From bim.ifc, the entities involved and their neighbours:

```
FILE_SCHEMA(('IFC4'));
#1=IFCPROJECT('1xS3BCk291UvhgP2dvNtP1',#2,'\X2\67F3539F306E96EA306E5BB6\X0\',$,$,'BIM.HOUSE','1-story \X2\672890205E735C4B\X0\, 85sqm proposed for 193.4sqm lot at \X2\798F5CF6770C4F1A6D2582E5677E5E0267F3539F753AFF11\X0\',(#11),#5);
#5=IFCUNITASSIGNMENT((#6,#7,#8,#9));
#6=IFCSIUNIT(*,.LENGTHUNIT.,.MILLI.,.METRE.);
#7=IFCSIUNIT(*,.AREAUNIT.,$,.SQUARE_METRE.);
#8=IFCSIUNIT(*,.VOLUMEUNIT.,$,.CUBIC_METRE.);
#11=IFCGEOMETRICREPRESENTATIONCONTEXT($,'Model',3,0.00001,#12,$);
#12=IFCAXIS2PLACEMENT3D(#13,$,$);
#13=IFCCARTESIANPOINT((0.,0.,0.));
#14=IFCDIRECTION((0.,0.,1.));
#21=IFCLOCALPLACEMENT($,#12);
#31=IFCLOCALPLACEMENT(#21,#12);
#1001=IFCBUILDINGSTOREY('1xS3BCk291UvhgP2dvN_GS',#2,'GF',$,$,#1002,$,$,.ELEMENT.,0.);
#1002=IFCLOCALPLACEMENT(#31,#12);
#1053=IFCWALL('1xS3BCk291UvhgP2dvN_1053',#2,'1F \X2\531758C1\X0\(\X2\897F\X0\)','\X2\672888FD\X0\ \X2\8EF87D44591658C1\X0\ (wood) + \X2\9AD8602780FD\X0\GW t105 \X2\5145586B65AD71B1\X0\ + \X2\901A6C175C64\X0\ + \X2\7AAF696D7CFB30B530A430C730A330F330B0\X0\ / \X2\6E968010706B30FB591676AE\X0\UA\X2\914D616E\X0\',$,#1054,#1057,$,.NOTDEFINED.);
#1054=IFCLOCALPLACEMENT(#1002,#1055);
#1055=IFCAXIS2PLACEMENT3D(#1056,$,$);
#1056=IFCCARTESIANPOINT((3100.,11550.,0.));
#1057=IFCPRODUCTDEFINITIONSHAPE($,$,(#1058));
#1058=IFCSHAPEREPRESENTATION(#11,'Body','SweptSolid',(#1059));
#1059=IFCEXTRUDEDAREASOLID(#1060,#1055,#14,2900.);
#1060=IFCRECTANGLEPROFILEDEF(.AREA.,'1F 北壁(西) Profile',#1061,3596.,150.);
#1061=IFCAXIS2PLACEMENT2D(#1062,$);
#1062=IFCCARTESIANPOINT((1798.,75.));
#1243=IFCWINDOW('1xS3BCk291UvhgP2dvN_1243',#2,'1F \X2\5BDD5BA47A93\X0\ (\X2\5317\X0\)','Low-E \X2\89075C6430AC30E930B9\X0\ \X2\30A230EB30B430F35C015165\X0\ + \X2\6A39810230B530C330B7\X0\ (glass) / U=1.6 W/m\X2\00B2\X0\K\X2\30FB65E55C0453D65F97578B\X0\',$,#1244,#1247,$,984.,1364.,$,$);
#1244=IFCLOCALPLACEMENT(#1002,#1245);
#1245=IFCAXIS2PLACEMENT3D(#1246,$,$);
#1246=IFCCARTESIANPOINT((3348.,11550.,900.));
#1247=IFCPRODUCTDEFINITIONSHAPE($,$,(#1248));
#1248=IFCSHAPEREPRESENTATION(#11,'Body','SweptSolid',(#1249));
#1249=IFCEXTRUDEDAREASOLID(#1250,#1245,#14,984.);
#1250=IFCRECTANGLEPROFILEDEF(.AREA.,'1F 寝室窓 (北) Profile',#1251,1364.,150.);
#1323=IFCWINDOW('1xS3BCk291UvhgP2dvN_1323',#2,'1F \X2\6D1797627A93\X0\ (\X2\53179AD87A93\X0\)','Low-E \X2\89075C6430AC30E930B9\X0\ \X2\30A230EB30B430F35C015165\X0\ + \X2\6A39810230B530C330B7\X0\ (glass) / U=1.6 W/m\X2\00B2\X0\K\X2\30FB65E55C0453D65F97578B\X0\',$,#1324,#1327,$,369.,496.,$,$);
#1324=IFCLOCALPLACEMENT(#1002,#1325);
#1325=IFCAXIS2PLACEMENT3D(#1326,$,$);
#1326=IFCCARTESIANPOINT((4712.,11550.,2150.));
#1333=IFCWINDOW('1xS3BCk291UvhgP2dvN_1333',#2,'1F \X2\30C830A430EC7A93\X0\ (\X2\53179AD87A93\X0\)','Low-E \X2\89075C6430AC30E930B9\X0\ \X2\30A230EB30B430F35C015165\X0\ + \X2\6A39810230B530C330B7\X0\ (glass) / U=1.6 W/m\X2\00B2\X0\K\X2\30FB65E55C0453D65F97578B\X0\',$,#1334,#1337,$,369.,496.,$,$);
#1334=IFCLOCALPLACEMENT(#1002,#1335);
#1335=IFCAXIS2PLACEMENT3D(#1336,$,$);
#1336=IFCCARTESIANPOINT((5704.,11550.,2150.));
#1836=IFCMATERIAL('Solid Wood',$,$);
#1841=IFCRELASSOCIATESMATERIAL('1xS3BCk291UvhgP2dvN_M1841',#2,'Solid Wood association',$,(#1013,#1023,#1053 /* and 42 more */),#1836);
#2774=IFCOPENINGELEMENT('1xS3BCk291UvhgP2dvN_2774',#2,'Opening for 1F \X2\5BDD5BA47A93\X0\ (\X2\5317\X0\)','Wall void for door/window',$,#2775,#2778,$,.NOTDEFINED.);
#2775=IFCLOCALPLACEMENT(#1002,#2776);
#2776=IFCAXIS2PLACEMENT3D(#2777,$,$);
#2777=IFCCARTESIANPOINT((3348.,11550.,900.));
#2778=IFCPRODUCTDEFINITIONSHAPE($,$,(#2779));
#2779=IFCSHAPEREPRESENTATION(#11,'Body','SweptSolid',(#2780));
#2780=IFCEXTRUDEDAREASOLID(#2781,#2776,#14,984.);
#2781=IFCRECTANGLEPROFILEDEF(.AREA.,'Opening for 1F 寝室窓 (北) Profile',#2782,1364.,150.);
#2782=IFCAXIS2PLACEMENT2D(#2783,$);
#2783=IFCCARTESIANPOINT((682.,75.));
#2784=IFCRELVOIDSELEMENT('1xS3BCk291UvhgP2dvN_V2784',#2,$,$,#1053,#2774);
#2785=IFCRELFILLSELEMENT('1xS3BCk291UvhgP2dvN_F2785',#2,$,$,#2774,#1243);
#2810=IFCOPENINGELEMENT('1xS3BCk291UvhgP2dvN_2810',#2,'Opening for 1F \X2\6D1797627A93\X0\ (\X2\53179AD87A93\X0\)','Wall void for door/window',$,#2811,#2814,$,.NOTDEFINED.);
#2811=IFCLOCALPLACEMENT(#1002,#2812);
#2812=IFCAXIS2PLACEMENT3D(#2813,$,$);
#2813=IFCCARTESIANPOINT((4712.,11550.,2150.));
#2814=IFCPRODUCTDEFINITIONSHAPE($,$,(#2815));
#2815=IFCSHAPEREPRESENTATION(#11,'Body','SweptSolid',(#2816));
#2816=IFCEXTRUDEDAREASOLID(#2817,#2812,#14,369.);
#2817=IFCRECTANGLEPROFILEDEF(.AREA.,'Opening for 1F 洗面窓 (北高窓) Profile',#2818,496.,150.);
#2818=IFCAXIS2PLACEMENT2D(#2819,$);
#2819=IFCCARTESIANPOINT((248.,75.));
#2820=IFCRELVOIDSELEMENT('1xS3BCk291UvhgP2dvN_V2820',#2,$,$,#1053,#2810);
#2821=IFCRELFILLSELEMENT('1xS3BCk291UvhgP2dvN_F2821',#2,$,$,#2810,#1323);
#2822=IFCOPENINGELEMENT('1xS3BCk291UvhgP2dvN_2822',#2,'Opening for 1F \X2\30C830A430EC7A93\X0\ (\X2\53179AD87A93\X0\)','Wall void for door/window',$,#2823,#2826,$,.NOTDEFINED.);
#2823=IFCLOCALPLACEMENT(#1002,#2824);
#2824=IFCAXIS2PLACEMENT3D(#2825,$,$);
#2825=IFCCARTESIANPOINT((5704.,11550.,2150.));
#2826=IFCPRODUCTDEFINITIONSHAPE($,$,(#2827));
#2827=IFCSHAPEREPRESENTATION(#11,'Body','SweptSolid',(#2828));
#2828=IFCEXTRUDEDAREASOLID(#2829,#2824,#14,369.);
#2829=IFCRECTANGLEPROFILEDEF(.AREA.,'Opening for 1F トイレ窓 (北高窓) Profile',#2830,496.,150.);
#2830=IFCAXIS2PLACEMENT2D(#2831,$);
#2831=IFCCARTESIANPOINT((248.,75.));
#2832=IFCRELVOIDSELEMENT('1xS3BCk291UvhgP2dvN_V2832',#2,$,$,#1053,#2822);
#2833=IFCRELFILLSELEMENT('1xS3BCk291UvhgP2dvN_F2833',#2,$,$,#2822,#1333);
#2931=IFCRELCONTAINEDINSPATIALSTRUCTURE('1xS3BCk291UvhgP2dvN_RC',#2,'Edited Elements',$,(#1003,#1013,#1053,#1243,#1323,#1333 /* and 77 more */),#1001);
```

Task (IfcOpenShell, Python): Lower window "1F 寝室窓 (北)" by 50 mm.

```python
import numpy as np
import ifcopenshell
import ifcopenshell.api.geometry
import ifcopenshell.util.placement
import ifcopenshell.util.unit

model = ifcopenshell.open("bim.ifc")
unit_scale = ifcopenshell.util.unit.calculate_unit_scale(model)

window = model.by_guid("1xS3BCk291UvhgP2dvN_1243")
opening = window.FillsVoids[0].RelatingOpeningElement
dz = -0.05 / unit_scale

shift = np.array([0.0, 0.0, dz])
# The window is not placed relative to its opening, so move both.
for product in (opening, window):
    matrix = ifcopenshell.util.placement.get_local_placement(product.ObjectPlacement)
    matrix[:3, 3] += shift
    ifcopenshell.api.geometry.edit_object_placement(model, product=product, matrix=matrix, is_si=False)

print(f"moved by {dz * unit_scale:+.3f} m")

model.write("bim_rev.ifc")
```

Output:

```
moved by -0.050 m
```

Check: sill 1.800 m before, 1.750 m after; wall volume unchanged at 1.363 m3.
